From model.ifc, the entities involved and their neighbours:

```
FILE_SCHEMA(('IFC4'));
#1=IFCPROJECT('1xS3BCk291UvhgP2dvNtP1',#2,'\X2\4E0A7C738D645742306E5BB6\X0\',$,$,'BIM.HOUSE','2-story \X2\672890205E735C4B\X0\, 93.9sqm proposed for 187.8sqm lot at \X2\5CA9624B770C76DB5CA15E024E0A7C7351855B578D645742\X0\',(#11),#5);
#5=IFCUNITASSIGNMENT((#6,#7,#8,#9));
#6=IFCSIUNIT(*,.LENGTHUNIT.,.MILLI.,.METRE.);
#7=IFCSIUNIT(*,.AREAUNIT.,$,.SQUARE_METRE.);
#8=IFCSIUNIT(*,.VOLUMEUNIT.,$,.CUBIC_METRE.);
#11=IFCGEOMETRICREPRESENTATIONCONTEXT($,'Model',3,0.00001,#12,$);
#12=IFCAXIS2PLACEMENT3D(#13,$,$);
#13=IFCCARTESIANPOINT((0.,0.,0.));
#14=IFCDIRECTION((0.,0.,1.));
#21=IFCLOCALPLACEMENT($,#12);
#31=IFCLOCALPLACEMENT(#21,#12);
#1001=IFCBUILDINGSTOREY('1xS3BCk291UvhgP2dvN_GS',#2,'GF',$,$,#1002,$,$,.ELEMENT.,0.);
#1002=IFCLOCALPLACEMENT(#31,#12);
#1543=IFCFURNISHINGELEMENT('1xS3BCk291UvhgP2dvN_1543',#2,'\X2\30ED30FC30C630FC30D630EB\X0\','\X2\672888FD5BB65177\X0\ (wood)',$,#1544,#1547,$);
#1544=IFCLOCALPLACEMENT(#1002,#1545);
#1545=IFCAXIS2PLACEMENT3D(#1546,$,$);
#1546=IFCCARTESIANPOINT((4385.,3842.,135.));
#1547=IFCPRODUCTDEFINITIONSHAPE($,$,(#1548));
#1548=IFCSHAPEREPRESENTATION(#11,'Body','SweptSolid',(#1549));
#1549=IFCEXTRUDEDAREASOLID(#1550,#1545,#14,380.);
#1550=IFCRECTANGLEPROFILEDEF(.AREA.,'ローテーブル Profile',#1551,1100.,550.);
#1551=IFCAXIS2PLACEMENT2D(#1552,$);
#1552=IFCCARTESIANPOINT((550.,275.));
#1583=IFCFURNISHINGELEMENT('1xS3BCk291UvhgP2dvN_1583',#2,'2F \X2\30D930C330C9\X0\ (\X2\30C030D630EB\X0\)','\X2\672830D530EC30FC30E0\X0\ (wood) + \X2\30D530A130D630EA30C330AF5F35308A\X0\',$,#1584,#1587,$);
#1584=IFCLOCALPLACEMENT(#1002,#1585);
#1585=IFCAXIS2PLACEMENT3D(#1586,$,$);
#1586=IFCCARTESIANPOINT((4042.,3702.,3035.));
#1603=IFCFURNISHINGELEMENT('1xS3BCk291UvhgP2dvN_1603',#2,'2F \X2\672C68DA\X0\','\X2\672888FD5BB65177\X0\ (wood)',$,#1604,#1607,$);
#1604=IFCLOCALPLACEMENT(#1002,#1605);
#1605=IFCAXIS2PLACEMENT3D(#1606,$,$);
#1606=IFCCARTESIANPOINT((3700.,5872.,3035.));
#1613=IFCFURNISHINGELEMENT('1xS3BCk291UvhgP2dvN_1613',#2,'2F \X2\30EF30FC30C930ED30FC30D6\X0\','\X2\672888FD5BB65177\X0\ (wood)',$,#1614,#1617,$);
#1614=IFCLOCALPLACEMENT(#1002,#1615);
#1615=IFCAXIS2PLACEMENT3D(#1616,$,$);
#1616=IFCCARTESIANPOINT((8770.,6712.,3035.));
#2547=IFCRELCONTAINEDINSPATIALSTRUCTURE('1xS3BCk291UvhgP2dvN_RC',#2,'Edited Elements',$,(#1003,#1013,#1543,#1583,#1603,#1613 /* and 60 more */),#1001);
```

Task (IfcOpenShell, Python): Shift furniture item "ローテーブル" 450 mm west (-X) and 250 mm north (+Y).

```python
import ifcopenshell
import ifcopenshell.api.geometry
import ifcopenshell.util.placement

model = ifcopenshell.open("model.ifc")

item = model.by_guid("1xS3BCk291UvhgP2dvN_1543")
matrix = ifcopenshell.util.placement.get_local_placement(item.ObjectPlacement)
matrix[0, 3] -= 450.0
matrix[1, 3] += 250.0
ifcopenshell.api.geometry.edit_object_placement(model, product=item, matrix=matrix, is_si=False)

print(ifcopenshell.util.placement.get_local_placement(item.ObjectPlacement).round(3) + 0.0)

model.write("model-out.ifc")
```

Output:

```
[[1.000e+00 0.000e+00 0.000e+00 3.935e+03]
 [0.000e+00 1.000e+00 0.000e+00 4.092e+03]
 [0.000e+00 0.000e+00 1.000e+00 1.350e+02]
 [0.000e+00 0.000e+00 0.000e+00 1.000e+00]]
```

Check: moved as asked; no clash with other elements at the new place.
